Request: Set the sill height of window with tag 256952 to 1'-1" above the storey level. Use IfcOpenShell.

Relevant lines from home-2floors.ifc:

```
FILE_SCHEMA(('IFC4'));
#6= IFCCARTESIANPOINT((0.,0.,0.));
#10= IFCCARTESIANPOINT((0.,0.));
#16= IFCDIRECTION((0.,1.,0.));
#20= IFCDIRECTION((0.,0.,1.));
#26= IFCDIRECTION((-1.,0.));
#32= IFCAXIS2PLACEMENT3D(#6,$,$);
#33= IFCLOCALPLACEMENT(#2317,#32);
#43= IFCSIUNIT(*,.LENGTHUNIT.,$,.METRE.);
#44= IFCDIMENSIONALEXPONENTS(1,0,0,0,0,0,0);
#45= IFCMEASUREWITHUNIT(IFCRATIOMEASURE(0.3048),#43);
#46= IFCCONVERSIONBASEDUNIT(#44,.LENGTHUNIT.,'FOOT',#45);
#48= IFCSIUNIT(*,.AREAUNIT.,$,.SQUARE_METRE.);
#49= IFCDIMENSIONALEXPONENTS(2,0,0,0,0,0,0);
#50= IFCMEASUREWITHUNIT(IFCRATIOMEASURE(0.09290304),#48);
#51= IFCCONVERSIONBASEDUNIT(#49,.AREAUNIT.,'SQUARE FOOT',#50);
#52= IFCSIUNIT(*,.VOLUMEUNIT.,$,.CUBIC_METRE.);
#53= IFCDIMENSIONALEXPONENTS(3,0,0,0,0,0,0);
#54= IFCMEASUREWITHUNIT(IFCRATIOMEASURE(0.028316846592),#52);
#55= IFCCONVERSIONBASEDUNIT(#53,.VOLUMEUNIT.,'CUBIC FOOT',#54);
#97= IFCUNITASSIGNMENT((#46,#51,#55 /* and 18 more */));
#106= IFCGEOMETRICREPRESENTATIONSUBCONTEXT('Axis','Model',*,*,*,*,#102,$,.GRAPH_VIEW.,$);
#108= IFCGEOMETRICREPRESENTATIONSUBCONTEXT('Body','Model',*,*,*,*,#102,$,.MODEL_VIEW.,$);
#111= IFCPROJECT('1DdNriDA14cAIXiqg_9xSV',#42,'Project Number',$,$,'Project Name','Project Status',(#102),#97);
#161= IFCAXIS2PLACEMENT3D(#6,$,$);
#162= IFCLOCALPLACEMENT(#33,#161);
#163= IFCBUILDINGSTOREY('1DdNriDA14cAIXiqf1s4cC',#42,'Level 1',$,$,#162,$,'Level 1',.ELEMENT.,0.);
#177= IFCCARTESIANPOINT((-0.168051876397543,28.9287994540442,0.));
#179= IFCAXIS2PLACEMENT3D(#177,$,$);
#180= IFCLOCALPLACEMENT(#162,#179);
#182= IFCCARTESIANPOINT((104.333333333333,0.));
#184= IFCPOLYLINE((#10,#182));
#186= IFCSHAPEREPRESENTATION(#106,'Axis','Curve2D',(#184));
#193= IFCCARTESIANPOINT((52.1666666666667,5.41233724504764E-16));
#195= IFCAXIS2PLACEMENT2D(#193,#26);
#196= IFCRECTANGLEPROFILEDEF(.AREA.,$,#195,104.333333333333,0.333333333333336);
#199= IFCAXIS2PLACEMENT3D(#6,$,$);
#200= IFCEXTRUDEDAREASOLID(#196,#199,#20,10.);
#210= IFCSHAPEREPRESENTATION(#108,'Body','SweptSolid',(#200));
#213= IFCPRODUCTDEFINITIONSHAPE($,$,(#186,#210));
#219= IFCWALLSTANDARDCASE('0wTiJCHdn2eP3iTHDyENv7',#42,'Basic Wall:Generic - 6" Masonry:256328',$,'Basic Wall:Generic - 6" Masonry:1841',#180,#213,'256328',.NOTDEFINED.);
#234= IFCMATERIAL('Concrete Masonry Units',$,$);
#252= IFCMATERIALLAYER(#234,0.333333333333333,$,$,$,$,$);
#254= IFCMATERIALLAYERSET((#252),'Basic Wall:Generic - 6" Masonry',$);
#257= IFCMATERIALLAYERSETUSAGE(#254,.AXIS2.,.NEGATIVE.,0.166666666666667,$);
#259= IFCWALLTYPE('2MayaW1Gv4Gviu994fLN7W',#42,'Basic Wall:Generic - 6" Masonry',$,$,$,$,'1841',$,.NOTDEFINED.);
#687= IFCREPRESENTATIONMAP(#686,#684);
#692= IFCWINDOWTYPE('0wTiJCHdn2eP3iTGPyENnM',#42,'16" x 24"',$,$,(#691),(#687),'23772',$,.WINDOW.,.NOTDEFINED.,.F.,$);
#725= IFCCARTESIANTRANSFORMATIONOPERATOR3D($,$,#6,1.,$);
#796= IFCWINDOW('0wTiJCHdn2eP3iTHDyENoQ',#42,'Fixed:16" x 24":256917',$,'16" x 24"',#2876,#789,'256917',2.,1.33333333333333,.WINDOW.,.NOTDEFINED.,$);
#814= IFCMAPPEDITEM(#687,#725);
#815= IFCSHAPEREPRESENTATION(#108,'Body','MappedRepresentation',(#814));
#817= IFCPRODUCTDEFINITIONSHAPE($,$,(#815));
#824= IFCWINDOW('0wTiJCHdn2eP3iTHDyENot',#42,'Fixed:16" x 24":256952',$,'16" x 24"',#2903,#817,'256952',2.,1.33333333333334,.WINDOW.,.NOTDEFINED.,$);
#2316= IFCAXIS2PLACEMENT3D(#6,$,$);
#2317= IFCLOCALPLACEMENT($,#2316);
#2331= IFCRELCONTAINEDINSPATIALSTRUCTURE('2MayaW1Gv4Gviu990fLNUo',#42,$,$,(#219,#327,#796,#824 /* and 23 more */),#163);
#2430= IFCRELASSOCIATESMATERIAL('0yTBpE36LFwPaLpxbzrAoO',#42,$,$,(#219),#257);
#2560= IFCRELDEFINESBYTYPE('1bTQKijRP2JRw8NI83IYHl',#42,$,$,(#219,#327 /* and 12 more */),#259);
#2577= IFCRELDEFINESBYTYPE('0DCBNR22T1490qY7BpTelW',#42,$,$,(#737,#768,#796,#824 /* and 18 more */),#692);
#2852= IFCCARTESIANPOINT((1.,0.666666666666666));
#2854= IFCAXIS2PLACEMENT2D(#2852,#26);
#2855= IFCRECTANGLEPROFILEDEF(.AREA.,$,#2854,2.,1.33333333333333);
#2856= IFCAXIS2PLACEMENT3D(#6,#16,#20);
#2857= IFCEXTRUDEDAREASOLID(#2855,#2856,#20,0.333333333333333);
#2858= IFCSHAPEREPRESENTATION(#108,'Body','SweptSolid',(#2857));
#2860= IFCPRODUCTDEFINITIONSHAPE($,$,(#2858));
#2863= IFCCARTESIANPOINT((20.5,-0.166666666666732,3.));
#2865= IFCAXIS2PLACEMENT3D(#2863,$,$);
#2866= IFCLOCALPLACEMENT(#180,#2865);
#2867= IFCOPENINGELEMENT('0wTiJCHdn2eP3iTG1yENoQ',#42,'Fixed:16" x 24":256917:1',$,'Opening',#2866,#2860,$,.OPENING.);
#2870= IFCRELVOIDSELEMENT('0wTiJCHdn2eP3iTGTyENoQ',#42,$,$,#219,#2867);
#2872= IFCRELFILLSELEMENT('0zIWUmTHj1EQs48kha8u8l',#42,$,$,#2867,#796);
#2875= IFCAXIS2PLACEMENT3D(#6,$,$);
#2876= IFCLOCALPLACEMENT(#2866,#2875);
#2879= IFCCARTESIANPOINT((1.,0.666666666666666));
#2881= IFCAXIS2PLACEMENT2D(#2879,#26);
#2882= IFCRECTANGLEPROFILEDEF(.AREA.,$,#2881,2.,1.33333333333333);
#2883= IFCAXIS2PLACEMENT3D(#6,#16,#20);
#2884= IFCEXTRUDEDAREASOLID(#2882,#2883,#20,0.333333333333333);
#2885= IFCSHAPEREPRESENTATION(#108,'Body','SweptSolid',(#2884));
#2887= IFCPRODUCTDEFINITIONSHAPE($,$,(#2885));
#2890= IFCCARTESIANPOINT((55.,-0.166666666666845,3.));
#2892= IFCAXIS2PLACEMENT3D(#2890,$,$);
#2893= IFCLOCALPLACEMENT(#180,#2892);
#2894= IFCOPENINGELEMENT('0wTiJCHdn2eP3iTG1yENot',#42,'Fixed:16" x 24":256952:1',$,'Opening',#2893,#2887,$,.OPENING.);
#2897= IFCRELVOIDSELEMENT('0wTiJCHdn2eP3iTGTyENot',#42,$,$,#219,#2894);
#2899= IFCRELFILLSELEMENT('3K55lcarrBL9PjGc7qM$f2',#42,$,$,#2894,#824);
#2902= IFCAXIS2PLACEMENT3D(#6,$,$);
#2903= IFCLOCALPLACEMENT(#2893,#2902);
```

```python
import numpy as np
import ifcopenshell
import ifcopenshell.api.geometry
import ifcopenshell.geom
import ifcopenshell.util.element
import ifcopenshell.util.placement
import ifcopenshell.util.shape
import ifcopenshell.util.unit

model = ifcopenshell.open("home-2floors.ifc")
unit_scale = ifcopenshell.util.unit.calculate_unit_scale(model)

window = model.by_id(824)
opening = window.FillsVoids[0].RelatingOpeningElement
storey = ifcopenshell.util.element.get_container(window, ifc_class="IfcBuildingStorey")
level = ifcopenshell.util.placement.get_local_placement(storey.ObjectPlacement)[2, 3]

# The opening's origin need not be at the sill, so measure its lowest point.
shape = ifcopenshell.geom.create_shape(ifcopenshell.geom.settings(), opening)
bottom = ifcopenshell.util.shape.get_shape_bottom_elevation(shape, shape.geometry) / unit_scale
dz = level + 13 * 0.0254 / unit_scale - bottom

shift = np.array([0.0, 0.0, dz])
# The window is placed relative to its opening, so it follows when the opening moves.
matrix = ifcopenshell.util.placement.get_local_placement(opening.ObjectPlacement)
matrix[:3, 3] += shift
ifcopenshell.api.geometry.edit_object_placement(
    model, product=opening, matrix=matrix, is_si=False, should_transform_children=True
)

print(f"moved by {dz * unit_scale:+.3f} m")

model.write("home-2floors-out.ifc")
```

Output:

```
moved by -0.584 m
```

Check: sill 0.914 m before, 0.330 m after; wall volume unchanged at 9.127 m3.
